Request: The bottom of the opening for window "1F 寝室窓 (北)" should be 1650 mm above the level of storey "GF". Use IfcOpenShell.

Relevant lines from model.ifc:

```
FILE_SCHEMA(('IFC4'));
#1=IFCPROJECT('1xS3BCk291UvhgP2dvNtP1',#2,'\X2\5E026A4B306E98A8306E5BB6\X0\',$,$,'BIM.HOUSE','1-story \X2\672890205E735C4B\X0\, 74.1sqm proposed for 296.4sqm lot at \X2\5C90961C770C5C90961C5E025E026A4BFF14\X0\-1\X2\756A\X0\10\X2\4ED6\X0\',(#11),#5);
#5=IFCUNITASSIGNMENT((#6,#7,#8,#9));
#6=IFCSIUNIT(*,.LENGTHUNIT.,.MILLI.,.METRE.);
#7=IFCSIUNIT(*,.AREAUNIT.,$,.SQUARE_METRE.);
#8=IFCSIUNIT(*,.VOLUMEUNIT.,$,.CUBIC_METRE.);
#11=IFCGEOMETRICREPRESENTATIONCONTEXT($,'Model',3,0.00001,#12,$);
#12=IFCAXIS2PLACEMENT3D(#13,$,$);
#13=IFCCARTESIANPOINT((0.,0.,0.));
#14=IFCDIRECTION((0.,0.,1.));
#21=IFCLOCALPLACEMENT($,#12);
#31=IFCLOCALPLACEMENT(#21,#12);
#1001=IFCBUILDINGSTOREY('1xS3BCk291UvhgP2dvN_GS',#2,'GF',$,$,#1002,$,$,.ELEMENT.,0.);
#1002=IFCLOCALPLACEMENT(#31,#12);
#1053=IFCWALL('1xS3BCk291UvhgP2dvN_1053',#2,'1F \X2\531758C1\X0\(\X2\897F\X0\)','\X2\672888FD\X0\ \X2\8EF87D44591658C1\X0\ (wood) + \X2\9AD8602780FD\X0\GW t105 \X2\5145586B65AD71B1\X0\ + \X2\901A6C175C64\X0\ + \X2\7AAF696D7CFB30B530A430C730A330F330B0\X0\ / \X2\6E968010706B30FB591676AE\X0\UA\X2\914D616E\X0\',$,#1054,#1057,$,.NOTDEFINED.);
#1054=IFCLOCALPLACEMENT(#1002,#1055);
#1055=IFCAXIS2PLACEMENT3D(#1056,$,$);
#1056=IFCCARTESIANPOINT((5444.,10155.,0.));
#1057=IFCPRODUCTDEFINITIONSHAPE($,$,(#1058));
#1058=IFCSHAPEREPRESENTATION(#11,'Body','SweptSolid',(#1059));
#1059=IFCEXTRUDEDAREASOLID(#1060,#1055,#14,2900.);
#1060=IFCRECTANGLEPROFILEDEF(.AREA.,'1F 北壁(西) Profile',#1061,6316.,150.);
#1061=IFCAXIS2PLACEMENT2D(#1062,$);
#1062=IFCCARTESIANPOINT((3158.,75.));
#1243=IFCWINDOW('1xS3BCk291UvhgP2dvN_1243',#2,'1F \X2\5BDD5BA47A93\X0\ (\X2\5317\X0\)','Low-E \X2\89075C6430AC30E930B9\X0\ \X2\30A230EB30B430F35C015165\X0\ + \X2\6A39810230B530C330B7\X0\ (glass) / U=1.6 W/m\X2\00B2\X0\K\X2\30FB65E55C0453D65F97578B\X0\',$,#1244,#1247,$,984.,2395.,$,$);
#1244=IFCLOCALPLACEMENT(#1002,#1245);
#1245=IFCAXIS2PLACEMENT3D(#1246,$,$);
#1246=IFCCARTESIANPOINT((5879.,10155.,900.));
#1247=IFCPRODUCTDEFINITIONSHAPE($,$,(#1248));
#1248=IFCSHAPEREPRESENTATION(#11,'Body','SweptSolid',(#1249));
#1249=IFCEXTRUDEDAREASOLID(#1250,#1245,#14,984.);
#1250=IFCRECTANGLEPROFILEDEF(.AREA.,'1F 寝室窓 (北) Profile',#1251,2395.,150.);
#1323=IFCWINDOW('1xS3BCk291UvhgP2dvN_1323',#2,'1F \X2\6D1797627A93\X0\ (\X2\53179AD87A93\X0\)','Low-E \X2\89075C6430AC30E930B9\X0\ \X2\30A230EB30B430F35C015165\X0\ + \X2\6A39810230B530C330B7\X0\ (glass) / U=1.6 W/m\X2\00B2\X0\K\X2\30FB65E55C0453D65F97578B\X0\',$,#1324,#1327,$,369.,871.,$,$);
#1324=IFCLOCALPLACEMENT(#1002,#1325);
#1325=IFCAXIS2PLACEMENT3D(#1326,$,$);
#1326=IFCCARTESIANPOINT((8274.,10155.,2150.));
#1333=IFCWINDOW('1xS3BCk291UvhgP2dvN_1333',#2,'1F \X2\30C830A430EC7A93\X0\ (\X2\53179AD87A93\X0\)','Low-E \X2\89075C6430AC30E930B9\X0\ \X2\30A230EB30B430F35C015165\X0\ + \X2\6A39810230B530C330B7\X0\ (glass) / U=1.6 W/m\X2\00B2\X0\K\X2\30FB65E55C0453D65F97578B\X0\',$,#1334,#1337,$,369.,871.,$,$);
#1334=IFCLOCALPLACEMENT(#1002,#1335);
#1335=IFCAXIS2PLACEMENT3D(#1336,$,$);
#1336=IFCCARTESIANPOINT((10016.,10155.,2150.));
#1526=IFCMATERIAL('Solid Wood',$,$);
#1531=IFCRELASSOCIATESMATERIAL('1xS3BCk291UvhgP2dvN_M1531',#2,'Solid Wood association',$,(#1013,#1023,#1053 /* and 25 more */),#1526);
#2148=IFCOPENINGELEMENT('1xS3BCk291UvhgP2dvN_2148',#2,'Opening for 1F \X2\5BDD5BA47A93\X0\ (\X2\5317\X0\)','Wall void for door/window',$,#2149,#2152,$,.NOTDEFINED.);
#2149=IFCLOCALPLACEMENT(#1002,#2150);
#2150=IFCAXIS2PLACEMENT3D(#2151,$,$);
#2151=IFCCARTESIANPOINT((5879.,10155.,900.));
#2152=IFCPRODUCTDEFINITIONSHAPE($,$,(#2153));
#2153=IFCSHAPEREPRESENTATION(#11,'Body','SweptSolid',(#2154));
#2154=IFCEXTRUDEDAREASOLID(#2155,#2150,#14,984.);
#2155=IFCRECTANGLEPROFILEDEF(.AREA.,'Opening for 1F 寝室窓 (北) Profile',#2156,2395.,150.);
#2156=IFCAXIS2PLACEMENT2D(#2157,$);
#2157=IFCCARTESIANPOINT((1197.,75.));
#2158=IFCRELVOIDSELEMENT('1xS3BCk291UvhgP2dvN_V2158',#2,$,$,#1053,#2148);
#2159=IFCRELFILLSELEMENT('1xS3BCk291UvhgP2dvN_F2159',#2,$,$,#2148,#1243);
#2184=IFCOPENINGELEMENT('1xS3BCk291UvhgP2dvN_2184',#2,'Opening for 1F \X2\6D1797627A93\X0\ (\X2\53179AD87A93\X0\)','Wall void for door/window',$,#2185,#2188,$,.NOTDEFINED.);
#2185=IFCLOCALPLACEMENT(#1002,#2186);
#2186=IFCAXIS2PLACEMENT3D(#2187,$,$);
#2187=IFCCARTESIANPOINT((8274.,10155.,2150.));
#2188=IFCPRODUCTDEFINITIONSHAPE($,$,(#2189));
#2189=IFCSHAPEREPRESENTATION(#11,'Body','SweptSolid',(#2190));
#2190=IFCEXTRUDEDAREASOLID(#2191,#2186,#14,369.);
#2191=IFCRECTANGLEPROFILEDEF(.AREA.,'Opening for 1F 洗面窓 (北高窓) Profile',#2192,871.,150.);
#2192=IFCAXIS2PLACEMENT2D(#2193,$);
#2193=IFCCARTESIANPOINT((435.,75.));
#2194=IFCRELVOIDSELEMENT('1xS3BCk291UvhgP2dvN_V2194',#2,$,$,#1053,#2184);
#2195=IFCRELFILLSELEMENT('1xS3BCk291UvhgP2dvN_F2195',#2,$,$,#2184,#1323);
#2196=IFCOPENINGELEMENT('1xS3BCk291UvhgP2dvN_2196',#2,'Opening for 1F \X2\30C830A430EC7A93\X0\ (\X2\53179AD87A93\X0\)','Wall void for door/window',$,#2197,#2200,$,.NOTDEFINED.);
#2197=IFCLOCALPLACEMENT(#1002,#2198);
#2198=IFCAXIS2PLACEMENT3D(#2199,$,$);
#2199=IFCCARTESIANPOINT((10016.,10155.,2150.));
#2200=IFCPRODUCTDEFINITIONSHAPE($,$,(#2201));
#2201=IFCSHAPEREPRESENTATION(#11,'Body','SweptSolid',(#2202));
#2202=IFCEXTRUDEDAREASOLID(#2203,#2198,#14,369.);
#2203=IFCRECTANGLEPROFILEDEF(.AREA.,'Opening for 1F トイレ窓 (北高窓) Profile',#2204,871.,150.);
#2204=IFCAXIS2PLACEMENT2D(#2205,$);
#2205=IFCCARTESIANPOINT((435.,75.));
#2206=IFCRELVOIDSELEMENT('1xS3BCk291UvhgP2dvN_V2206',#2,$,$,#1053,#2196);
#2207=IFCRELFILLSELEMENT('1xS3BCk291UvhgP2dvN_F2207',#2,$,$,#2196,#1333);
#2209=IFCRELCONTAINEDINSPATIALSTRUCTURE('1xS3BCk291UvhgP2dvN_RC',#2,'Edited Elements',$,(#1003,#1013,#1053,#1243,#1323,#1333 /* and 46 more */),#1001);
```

```python
import numpy as np
import ifcopenshell
import ifcopenshell.api.geometry
import ifcopenshell.geom
import ifcopenshell.util.element
import ifcopenshell.util.placement
import ifcopenshell.util.shape
import ifcopenshell.util.unit

model = ifcopenshell.open("model.ifc")
unit_scale = ifcopenshell.util.unit.calculate_unit_scale(model)

window = model.by_guid("1xS3BCk291UvhgP2dvN_1243")
opening = window.FillsVoids[0].RelatingOpeningElement
storey = ifcopenshell.util.element.get_container(window, ifc_class="IfcBuildingStorey")
level = ifcopenshell.util.placement.get_local_placement(storey.ObjectPlacement)[2, 3]

# The opening's origin need not be at the sill, so measure its lowest point.
shape = ifcopenshell.geom.create_shape(ifcopenshell.geom.settings(), opening)
bottom = ifcopenshell.util.shape.get_shape_bottom_elevation(shape, shape.geometry) / unit_scale
dz = level + 1.65 / unit_scale - bottom

shift = np.array([0.0, 0.0, dz])
# The window is not placed relative to its opening, so move both.
for product in (opening, window):
    matrix = ifcopenshell.util.placement.get_local_placement(product.ObjectPlacement)
    matrix[:3, 3] += shift
    ifcopenshell.api.geometry.edit_object_placement(model, product=product, matrix=matrix, is_si=False)

print(f"moved by {dz * unit_scale:+.3f} m")

model.write("model_updated.ifc")
```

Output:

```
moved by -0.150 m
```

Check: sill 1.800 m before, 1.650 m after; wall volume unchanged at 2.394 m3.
